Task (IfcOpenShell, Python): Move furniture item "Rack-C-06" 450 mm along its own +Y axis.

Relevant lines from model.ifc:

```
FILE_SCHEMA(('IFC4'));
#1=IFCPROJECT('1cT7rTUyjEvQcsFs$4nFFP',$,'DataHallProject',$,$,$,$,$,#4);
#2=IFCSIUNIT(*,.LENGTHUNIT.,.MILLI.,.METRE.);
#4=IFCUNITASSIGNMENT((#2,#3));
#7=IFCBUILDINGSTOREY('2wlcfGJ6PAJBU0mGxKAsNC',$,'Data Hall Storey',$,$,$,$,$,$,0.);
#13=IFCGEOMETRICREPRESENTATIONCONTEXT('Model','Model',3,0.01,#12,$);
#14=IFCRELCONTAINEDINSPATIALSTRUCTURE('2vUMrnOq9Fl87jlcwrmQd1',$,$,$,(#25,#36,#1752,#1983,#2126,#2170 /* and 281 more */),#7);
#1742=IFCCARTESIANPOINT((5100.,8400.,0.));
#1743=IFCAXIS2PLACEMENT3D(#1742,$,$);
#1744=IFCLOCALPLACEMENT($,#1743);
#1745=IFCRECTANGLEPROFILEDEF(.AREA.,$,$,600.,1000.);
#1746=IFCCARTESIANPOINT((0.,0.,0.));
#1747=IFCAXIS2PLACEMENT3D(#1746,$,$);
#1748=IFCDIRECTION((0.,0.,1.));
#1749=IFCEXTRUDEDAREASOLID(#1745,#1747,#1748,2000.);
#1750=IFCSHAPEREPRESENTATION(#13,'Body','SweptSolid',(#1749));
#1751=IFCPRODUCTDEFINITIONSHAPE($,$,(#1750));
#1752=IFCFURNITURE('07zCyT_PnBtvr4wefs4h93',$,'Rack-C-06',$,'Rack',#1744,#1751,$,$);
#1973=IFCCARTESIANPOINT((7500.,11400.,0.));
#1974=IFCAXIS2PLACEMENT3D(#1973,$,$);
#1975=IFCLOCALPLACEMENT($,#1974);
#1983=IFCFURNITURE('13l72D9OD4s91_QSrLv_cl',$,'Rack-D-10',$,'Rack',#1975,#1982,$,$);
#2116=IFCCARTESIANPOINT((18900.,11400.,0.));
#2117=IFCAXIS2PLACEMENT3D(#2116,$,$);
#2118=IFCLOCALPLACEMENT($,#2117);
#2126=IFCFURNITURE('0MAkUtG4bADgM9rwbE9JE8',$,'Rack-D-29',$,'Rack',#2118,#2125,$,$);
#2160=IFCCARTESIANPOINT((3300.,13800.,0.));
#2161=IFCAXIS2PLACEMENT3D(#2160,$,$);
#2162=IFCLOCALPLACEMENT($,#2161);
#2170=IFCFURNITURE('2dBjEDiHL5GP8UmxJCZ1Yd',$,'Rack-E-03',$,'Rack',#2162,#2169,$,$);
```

```python
import ifcopenshell
import ifcopenshell.api.geometry
import ifcopenshell.util.placement

model = ifcopenshell.open("model.ifc")

item = model.by_id(1752)
matrix = ifcopenshell.util.placement.get_local_placement(item.ObjectPlacement)
matrix[:3, 3] += matrix[:3, 1] * 450.0
ifcopenshell.api.geometry.edit_object_placement(model, product=item, matrix=matrix, is_si=False)

print(ifcopenshell.util.placement.get_local_placement(item.ObjectPlacement).round(3) + 0.0)

model.write("model_v2.ifc")
```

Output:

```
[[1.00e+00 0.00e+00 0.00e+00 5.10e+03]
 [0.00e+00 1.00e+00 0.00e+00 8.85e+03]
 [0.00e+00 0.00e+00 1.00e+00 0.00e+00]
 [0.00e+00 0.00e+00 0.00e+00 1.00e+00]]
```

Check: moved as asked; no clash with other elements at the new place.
